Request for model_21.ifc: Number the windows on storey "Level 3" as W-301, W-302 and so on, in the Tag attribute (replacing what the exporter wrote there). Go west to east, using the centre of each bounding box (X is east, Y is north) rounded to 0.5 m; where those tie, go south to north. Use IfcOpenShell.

First a look at what the model holds.

```python
import ifcopenshell
import ifcopenshell.util.element
import ifcopenshell.util.placement

model = ifcopenshell.open("model_21.ifc")
print(model.schema)
storey = next(s for s in model.by_type("IfcBuildingStorey") if s.Name == "Level 3")
windows = [e for e in ifcopenshell.util.element.get_decomposition(storey) if e.is_a("IfcWindow")]
for e in sorted(windows, key=lambda e: e.id()):
    origin = ifcopenshell.util.placement.get_local_placement(e.ObjectPlacement)[:3, 3]
    print(e.id(), e.Tag, e.Name, origin.round(2) + 0.0, sep=" | ")
```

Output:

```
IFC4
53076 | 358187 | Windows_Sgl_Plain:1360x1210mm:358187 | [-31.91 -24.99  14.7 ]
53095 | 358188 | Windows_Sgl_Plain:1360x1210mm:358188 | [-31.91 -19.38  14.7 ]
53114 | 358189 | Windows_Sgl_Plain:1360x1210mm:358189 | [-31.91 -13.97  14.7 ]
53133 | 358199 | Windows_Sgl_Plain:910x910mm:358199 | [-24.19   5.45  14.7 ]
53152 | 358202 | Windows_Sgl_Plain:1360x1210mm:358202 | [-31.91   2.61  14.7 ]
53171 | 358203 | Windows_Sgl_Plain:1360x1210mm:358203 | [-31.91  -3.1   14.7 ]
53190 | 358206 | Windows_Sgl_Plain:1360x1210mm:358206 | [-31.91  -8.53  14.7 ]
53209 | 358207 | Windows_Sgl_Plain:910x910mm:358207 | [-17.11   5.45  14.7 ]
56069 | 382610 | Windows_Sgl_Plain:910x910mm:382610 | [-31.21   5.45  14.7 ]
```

```python
import ifcopenshell
import ifcopenshell.geom
import ifcopenshell.util.element
import ifcopenshell.util.shape

model = ifcopenshell.open("model_21.ifc")
settings = ifcopenshell.geom.settings()
settings.set("use-world-coords", True)


def centre(element):
    shape = ifcopenshell.geom.create_shape(settings, element)
    return ifcopenshell.util.shape.get_bbox_centroid(shape.geometry)


storey = next(s for s in model.by_type("IfcBuildingStorey") if s.Name == "Level 3")
windows = [e for e in ifcopenshell.util.element.get_decomposition(storey) if e.is_a("IfcWindow")]

# Insertion points can sit at a corner or the storey origin, so sort by the geometry (in metres).
centres = {e: centre(e) for e in windows}
windows.sort(key=lambda e: (round(centres[e][0] / 0.5), centres[e][1]))

for i, e in enumerate(windows, start=1):
    number = f"W-3{i:02d}"
    e.Tag = number
    print(e.id(), number)

model.write("model_21_edited.ifc")
```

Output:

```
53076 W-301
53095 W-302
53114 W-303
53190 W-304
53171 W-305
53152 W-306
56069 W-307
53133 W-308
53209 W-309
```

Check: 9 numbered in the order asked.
